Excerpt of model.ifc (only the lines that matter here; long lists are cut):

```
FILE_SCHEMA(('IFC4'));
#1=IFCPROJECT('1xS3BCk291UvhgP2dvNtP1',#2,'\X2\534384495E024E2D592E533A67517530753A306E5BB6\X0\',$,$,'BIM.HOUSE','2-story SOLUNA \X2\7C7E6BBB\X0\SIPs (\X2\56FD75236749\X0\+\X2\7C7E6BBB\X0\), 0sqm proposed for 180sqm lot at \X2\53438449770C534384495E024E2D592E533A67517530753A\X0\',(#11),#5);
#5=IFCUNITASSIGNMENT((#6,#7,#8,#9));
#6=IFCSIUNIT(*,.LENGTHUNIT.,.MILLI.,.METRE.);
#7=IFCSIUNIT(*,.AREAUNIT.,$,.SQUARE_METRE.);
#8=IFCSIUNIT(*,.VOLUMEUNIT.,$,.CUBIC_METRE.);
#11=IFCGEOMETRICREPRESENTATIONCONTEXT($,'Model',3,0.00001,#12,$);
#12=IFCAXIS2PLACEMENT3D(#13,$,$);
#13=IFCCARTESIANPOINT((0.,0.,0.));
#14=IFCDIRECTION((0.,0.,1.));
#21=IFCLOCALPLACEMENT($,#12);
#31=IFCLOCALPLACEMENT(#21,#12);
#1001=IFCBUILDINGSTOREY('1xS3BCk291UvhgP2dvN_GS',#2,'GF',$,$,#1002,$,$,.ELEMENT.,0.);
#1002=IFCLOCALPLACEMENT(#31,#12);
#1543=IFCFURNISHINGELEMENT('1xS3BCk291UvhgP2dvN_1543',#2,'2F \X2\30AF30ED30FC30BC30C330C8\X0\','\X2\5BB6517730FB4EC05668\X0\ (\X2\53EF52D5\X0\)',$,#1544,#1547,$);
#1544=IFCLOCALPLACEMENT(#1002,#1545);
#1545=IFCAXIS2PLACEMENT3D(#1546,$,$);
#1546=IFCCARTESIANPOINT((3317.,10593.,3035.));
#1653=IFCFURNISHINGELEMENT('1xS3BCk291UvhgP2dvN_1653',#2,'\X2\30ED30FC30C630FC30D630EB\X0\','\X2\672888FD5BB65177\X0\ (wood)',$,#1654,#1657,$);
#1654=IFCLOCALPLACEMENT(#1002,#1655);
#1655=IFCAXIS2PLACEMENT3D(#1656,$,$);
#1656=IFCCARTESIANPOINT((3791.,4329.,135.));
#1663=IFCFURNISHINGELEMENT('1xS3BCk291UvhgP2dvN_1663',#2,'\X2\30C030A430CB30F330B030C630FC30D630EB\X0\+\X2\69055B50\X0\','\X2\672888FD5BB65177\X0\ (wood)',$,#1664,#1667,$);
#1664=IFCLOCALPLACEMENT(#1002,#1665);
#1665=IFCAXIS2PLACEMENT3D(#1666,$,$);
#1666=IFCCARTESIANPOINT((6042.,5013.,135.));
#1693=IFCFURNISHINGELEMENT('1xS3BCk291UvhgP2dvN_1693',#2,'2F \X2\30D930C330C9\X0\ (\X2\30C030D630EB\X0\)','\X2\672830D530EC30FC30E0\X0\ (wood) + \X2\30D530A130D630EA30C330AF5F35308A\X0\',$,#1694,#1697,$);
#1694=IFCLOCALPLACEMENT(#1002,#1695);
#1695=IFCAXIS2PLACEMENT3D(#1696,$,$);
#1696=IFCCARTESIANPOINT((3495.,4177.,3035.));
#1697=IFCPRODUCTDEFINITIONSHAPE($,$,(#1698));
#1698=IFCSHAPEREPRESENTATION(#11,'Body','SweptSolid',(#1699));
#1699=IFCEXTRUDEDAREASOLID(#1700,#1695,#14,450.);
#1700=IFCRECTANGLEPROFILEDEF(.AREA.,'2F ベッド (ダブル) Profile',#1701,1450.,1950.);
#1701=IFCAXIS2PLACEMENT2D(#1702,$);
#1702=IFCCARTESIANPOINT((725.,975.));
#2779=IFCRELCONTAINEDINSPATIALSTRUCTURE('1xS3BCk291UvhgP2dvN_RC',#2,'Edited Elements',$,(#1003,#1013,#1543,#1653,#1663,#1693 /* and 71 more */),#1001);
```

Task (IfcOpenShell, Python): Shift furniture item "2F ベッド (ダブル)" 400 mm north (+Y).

```python
import ifcopenshell
import ifcopenshell.api.geometry
import ifcopenshell.util.placement
import ifcopenshell.util.unit

model = ifcopenshell.open("model.ifc")
unit_scale = ifcopenshell.util.unit.calculate_unit_scale(model)

item = model.by_id(1693)
matrix = ifcopenshell.util.placement.get_local_placement(item.ObjectPlacement)
matrix[1, 3] += 0.4 / unit_scale
ifcopenshell.api.geometry.edit_object_placement(model, product=item, matrix=matrix, is_si=False)

print(ifcopenshell.util.placement.get_local_placement(item.ObjectPlacement).round(3) + 0.0)

model.write("model_updated.ifc")
```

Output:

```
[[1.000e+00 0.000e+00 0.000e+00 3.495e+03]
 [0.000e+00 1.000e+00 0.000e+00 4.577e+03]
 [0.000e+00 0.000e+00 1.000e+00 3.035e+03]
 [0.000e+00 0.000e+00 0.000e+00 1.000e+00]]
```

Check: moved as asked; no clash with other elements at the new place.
